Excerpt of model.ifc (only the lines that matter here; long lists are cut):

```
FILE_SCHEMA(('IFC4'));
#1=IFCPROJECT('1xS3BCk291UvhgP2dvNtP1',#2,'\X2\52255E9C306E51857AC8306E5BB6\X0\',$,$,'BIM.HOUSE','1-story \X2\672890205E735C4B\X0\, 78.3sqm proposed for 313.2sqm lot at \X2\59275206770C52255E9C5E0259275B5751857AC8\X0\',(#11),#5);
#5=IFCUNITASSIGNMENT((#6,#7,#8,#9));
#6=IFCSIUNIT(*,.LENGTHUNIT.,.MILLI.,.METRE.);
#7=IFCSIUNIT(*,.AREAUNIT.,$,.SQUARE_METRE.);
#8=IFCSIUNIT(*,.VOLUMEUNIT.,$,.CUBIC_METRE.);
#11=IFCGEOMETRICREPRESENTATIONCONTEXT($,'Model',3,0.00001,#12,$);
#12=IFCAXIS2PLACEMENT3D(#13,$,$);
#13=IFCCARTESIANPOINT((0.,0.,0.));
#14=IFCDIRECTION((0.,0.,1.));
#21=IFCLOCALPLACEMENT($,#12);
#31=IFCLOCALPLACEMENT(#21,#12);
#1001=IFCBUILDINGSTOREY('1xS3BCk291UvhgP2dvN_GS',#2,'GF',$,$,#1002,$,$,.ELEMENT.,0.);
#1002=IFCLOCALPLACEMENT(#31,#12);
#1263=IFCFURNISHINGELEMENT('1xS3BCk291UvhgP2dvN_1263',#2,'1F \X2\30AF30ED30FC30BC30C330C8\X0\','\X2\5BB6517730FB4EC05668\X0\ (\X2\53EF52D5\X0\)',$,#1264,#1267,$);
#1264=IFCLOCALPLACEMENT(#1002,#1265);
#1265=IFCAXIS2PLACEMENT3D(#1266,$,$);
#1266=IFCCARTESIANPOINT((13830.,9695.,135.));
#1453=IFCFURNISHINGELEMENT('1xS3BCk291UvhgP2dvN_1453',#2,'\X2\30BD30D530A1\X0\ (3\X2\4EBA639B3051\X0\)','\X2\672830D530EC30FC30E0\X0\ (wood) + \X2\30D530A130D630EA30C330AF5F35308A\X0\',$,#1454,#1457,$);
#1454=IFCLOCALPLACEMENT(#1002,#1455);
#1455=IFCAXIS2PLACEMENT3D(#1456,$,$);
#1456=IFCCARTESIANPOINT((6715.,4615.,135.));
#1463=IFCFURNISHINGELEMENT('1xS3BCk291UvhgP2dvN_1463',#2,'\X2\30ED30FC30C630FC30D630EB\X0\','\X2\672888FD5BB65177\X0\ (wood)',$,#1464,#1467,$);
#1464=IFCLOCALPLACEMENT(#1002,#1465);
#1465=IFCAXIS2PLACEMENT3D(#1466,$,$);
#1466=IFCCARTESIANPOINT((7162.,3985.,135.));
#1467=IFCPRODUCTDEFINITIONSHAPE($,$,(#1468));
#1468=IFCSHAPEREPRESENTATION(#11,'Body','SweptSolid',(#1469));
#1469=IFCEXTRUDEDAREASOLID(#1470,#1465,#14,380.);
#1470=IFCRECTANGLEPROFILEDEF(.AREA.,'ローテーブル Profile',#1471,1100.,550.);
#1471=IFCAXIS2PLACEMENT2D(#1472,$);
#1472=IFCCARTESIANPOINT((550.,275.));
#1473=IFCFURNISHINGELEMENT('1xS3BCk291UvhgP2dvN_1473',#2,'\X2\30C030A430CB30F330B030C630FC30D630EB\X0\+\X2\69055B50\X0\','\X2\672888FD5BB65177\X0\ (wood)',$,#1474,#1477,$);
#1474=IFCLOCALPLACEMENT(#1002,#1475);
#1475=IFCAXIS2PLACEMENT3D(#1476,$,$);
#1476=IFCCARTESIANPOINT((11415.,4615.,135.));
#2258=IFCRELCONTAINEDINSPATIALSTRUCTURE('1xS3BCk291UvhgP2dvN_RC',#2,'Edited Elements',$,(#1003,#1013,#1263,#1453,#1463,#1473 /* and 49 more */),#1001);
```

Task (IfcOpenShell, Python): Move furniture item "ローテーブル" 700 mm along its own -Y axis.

```python
import ifcopenshell
import ifcopenshell.api.geometry
import ifcopenshell.util.placement
import ifcopenshell.util.unit

model = ifcopenshell.open("model.ifc")
unit_scale = ifcopenshell.util.unit.calculate_unit_scale(model)

item = model.by_id(1463)
matrix = ifcopenshell.util.placement.get_local_placement(item.ObjectPlacement)
matrix[:3, 3] -= matrix[:3, 1] * 0.7 / unit_scale
ifcopenshell.api.geometry.edit_object_placement(model, product=item, matrix=matrix, is_si=False)

print(ifcopenshell.util.placement.get_local_placement(item.ObjectPlacement).round(3) + 0.0)

model.write("model-out.ifc")
```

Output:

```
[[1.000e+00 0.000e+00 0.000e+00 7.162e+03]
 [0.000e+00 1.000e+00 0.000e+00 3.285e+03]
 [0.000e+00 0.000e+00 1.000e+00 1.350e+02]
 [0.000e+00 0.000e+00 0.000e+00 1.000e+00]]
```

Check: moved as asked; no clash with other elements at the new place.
